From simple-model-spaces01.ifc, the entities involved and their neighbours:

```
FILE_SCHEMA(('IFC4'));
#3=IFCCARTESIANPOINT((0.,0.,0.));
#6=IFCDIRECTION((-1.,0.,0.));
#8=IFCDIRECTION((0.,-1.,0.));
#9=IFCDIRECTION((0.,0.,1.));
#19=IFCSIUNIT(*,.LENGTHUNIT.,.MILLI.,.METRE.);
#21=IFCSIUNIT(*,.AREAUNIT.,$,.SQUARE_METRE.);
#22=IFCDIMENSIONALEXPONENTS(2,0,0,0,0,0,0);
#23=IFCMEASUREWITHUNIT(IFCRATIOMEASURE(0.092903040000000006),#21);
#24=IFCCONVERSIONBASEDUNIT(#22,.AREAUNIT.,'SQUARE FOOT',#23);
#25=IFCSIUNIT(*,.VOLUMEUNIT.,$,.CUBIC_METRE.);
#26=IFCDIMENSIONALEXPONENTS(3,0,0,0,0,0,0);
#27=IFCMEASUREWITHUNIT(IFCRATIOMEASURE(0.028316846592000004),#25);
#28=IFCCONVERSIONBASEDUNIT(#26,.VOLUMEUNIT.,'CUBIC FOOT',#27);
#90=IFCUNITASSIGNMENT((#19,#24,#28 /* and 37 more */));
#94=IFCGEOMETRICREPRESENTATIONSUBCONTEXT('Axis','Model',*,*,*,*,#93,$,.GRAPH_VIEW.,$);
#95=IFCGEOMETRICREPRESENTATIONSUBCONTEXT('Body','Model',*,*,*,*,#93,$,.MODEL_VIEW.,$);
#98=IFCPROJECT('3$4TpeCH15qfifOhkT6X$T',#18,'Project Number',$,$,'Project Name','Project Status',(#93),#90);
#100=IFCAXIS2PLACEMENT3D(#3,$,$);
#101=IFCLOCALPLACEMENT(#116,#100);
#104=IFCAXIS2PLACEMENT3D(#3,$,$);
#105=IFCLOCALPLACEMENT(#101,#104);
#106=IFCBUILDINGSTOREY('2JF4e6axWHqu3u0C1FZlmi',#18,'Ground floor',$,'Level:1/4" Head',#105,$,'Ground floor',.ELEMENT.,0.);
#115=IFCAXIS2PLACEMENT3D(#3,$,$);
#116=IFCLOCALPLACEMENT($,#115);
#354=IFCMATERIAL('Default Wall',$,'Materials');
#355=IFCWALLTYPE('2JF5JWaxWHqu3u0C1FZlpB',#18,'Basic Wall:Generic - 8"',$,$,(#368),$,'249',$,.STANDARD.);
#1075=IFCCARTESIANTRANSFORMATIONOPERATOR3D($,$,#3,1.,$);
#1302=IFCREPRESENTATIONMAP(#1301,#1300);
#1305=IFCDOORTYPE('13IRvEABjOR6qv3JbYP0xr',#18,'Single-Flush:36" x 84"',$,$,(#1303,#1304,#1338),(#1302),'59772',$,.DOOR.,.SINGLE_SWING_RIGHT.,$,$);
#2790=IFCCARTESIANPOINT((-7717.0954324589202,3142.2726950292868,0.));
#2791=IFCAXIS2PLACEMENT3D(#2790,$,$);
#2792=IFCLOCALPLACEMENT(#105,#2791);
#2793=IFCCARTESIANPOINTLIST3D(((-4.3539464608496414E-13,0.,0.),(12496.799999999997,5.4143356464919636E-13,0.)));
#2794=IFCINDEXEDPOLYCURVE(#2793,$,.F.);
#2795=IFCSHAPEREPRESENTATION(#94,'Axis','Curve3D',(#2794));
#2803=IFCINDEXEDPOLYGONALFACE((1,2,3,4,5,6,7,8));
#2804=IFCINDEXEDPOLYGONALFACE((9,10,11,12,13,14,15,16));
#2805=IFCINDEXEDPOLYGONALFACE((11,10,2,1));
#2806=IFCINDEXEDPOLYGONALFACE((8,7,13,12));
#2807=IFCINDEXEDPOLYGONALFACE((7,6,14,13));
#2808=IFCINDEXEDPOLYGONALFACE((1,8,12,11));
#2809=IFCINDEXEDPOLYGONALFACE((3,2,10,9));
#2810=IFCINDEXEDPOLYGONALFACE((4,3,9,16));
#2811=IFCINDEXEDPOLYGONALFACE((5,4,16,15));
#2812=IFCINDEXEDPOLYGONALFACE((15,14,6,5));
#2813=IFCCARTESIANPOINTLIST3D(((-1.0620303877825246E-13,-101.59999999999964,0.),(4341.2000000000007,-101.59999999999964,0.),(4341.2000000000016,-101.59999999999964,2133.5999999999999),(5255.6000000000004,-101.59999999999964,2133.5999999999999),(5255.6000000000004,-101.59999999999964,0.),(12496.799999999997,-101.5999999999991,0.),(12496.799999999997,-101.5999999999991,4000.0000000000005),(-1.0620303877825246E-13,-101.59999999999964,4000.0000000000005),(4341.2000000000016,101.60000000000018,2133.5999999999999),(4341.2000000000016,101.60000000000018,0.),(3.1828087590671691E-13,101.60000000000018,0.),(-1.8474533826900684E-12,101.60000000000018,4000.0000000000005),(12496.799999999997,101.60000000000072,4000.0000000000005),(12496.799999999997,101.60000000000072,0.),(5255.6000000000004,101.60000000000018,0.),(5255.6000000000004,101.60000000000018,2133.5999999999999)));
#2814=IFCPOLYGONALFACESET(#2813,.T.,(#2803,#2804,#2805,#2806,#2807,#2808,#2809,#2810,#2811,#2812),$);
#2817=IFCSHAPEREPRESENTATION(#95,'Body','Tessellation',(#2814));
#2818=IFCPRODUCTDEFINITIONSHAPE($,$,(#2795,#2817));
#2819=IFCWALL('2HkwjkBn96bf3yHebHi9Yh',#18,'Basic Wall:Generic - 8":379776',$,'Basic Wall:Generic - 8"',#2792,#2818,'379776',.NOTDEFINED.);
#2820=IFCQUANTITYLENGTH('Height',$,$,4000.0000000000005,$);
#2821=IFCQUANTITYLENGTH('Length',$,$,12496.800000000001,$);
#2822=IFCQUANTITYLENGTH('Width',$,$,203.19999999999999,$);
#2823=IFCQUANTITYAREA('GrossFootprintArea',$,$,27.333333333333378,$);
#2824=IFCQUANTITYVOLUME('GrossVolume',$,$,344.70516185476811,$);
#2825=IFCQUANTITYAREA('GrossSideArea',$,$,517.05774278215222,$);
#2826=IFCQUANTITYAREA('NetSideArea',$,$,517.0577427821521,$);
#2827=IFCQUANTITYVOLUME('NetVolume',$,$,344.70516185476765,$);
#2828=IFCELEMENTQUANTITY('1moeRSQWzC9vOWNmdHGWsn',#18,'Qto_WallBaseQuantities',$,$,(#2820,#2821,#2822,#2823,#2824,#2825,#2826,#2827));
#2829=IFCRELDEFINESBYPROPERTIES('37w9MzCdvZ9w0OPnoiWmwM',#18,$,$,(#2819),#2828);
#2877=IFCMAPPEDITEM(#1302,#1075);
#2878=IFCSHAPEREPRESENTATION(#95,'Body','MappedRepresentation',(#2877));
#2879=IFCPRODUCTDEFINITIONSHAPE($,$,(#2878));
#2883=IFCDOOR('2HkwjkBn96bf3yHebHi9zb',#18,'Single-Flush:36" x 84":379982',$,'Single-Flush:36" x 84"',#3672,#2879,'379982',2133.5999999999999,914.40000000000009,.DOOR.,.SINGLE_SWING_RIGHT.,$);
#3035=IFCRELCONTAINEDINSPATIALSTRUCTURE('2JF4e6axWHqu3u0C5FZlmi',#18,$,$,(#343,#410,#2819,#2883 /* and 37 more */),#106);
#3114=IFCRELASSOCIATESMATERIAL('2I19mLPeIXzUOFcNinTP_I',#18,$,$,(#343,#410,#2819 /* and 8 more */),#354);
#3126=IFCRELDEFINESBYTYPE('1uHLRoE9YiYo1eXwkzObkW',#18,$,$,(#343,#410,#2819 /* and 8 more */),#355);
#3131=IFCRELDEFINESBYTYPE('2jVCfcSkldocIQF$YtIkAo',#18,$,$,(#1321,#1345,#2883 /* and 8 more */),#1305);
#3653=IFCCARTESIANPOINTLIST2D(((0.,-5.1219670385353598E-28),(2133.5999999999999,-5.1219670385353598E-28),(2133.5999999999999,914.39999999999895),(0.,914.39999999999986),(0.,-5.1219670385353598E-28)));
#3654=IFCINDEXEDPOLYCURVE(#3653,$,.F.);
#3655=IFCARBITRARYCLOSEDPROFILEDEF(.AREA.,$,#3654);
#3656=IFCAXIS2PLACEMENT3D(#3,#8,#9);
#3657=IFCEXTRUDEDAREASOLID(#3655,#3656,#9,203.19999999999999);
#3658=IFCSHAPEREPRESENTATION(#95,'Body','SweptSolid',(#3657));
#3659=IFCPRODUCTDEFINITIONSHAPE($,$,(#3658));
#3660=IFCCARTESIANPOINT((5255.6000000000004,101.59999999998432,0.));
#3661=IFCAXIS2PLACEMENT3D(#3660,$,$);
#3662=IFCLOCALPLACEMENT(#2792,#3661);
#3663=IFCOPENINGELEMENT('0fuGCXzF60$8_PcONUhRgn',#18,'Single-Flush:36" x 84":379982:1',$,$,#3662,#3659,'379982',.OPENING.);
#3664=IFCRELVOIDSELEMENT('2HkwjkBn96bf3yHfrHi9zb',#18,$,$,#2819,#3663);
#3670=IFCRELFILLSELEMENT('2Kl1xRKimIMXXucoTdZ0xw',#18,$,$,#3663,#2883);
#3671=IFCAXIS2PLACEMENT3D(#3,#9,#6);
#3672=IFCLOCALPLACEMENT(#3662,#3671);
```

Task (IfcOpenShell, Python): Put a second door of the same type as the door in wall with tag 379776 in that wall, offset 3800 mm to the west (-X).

```python
import ifcopenshell
import ifcopenshell.api.feature
import ifcopenshell.api.geometry
import ifcopenshell.api.pset
import ifcopenshell.api.root
import ifcopenshell.geom
import ifcopenshell.util.element
import ifcopenshell.util.placement
import ifcopenshell.util.shape
import ifcopenshell.util.unit

model = ifcopenshell.open("simple-model-spaces01.ifc")
area_scale = ifcopenshell.util.unit.calculate_unit_scale(model, "AREAUNIT")
volume_scale = ifcopenshell.util.unit.calculate_unit_scale(model, "VOLUMEUNIT")
settings = ifcopenshell.geom.settings()


def volume(element):
    """Net volume in cubic metres, openings subtracted."""
    shape = ifcopenshell.geom.create_shape(settings, element)
    return ifcopenshell.util.shape.get_volume(shape.geometry)


def reuse_history(source, copy):
    """copy_class also copies each property set's owner history, people and application; keep the originals."""
    for rel in copy.IsDefinedBy:
        if rel.is_a("IfcRelDefinesByProperties") and (history := rel.RelatingPropertyDefinition.OwnerHistory):
            rel.RelatingPropertyDefinition.OwnerHistory = source.OwnerHistory
            ifcopenshell.util.element.remove_deep2(model, history)


door = model.by_id(2883)
opening = door.FillsVoids[0].RelatingOpeningElement
wall = opening.VoidsElements[0].RelatingBuildingElement
before = volume(wall)
shift = ifcopenshell.util.placement.get_local_placement(wall.ObjectPlacement)[:3, 0] * -3800.0

# copy_class copies the void relationship, type, container and properties, but no geometry.
new_opening = ifcopenshell.api.root.copy_class(model, product=opening)
new_opening.Representation = ifcopenshell.util.element.copy_deep(
    model, opening.Representation, exclude=["IfcGeometricRepresentationContext", "IfcRepresentationMap"]
)
new_opening.Name = 'Single-Flush:36" x 84"'
new_opening.Tag = None
reuse_history(opening, new_opening)
new_door = ifcopenshell.api.root.copy_class(model, product=door)
new_door.Representation = ifcopenshell.util.element.copy_deep(
    model, door.Representation, exclude=["IfcGeometricRepresentationContext", "IfcRepresentationMap"]
)
new_door.Name = 'Single-Flush:36" x 84"'
new_door.Tag = None
reuse_history(door, new_door)
ifcopenshell.api.feature.add_filling(model, opening=new_opening, element=new_door)

for old, new in ((opening, new_opening), (door, new_door)):
    matrix = ifcopenshell.util.placement.get_local_placement(old.ObjectPlacement)
    matrix[:3, 3] += shift
    ifcopenshell.api.geometry.edit_object_placement(model, product=new, matrix=matrix, is_si=False)

after = volume(wall)
thickness = 0.2032  # wall thickness in metres

# Update the wall's stored quantities.
qto = model.by_id(ifcopenshell.util.element.get_pset(wall, "Qto_WallBaseQuantities", should_inherit=False)["id"])
ifcopenshell.api.pset.edit_qto(model, qto=qto, properties={
    "NetSideArea": after / thickness / area_scale,
    "NetVolume": after / volume_scale,
})

print(f"wall volume {before:.3f} -> {after:.3f} m3")

model.write("simple-model-spaces01_edited.ifc")
```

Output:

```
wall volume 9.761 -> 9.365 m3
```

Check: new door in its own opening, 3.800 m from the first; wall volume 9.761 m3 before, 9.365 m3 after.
